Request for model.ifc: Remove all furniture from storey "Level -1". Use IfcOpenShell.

First a look at what the model holds.

```python
import ifcopenshell
import ifcopenshell.util.element

model = ifcopenshell.open("model.ifc")
print(model.schema)
storey = next(s for s in model.by_type("IfcBuildingStorey") if s.Name == "Level -1")
furniture = [e for e in ifcopenshell.util.element.get_decomposition(storey) if e.is_a("IfcFurnishingElement")]
seen = {}
for e in furniture:
    element_type = ifcopenshell.util.element.get_type(e)
    name = element_type.Name if element_type not in (None, e) else None
    seen[name] = seen.get(name, 0) + 1
for name, count in sorted(seen.items(), key=str):
    print(count, "x", name)
```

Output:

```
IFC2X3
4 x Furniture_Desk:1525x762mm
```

```python
import ifcopenshell
import ifcopenshell.api.root
import ifcopenshell.util.element

model = ifcopenshell.open("model.ifc")

storey = next(s for s in model.by_type("IfcBuildingStorey") if s.Name == "Level -1")
furniture = [e for e in ifcopenshell.util.element.get_decomposition(storey) if e.is_a("IfcFurnishingElement")]

for e in furniture:
    ifcopenshell.api.root.remove_product(model, product=e)
print(len(furniture), "removed")

model.write("model-out.ifc")
```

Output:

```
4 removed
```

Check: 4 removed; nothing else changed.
